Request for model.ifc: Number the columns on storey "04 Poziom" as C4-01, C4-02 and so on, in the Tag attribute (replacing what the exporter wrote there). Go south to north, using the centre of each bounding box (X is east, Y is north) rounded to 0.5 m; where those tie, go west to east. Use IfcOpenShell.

First a look at what the model holds.

```python
import ifcopenshell
import ifcopenshell.util.element
import ifcopenshell.util.placement

model = ifcopenshell.open("model.ifc")
print(model.schema)
storey = next(s for s in model.by_type("IfcBuildingStorey") if s.Name == "04 Poziom")
columns = [e for e in ifcopenshell.util.element.get_decomposition(storey) if e.is_a("IfcColumn")]
for e in sorted(columns, key=lambda e: e.id()):
    origin = ifcopenshell.util.placement.get_local_placement(e.ObjectPlacement)[:3, 3]
    print(e.id(), e.Tag, e.Name, origin.round(2) + 0.0, sep=" | ")
```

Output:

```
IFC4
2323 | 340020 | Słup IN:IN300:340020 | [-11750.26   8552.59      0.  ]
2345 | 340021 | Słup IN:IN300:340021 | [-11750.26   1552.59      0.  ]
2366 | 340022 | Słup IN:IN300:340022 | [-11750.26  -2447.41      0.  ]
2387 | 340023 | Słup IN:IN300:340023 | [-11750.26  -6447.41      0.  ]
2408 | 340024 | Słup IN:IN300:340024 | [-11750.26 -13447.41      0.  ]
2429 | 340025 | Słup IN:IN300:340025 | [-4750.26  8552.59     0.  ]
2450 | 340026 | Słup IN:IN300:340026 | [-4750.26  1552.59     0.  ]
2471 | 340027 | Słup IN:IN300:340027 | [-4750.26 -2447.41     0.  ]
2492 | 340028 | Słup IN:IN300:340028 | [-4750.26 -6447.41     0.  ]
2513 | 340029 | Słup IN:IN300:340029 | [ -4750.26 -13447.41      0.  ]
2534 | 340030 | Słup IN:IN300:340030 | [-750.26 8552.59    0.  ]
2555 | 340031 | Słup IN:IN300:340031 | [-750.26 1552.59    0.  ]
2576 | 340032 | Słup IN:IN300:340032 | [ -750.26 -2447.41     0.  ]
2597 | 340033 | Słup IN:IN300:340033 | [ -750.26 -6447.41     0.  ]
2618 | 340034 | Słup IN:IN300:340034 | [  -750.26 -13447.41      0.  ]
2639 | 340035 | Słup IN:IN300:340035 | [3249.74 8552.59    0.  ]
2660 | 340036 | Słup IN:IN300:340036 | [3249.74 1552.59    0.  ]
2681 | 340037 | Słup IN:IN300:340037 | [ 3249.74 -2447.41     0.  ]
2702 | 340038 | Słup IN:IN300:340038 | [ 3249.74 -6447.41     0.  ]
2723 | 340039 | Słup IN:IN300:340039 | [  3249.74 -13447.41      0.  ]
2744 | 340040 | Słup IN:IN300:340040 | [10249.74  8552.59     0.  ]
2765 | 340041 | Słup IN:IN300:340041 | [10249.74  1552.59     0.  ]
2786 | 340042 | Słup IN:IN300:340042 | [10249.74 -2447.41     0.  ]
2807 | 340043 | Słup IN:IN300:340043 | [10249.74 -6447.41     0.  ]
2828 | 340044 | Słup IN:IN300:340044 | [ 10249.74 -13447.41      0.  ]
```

```python
import ifcopenshell
import ifcopenshell.geom
import ifcopenshell.util.element
import ifcopenshell.util.shape

model = ifcopenshell.open("model.ifc")
settings = ifcopenshell.geom.settings()
settings.set("use-world-coords", True)


def centre(element):
    shape = ifcopenshell.geom.create_shape(settings, element)
    return ifcopenshell.util.shape.get_bbox_centroid(shape.geometry)


storey = next(s for s in model.by_type("IfcBuildingStorey") if s.Name == "04 Poziom")
columns = [e for e in ifcopenshell.util.element.get_decomposition(storey) if e.is_a("IfcColumn")]

# Insertion points can sit at a corner or the storey origin, so sort by the geometry (in metres).
centres = {e: centre(e) for e in columns}
columns.sort(key=lambda e: (round(centres[e][1] / 0.5), centres[e][0]))

for i, e in enumerate(columns, start=1):
    number = f"C4-{i:02d}"
    e.Tag = number
    print(e.id(), number)

model.write("model_v2.ifc")
```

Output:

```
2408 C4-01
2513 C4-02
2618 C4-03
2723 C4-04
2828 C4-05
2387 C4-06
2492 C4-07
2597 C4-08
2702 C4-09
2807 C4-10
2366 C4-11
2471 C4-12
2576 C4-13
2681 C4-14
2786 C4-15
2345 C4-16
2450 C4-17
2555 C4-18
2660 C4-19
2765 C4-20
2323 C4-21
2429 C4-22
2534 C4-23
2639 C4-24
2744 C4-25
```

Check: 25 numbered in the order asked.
